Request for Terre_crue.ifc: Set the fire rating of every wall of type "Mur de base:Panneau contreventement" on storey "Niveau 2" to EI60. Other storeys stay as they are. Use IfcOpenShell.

First a look at what the model holds.

```python
import ifcopenshell
import ifcopenshell.util.element

model = ifcopenshell.open("Terre_crue.ifc")
print(model.schema)
storey = next(s for s in model.by_type("IfcBuildingStorey") if s.Name == "Niveau 2")
walls = [e for e in ifcopenshell.util.element.get_decomposition(storey) if e.is_a("IfcWall")]
seen = {}
for e in walls:
    element_type = ifcopenshell.util.element.get_type(e)
    key = (element_type.Name if element_type != e and element_type else None, ifcopenshell.util.element.get_pset(e, "Pset_WallCommon", "FireRating"))
    seen[key] = seen.get(key, 0) + 1
for (name, value), count in sorted(seen.items(), key=str):
    print(count, "x", name, "|", value)
```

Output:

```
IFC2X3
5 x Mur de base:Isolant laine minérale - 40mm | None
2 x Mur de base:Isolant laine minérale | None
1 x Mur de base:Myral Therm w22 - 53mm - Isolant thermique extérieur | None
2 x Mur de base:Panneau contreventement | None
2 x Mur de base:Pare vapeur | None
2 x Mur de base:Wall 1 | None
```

```python
import ifcopenshell
import ifcopenshell.api.pset
import ifcopenshell.util.element

model = ifcopenshell.open("Terre_crue.ifc")

storey = next(s for s in model.by_type("IfcBuildingStorey") if s.Name == "Niveau 2")
walls = [e for e in ifcopenshell.util.element.get_decomposition(storey) if e.is_a("IfcWall")]

count = 0
for e in walls:
    element_type = ifcopenshell.util.element.get_type(e)
    if element_type in (None, e) or element_type.Name != "Mur de base:Panneau contreventement":
        continue
    # add_pset returns the element's existing set when there is one.
    pset = ifcopenshell.api.pset.add_pset(model, product=e, name="Pset_WallCommon")
    ifcopenshell.api.pset.edit_pset(model, pset=pset, properties={"FireRating": "EI60"})
    count += 1

print(count, "walls updated")

model.write("Terre_crue_edited.ifc")
```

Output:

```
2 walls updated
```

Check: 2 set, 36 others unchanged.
